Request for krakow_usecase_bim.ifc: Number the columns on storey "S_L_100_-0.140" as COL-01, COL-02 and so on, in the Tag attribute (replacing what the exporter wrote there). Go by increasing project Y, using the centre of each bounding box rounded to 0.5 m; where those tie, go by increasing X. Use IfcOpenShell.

First a look at what the model holds.

```python
import ifcopenshell
import ifcopenshell.util.element
import ifcopenshell.util.placement

model = ifcopenshell.open("krakow_usecase_bim.ifc")
print(model.schema)
storey = next(s for s in model.by_type("IfcBuildingStorey") if s.Name == "S_L_100_-0.140")
columns = [e for e in ifcopenshell.util.element.get_decomposition(storey) if e.is_a("IfcColumn")]
for e in sorted(columns, key=lambda e: e.id()):
    origin = ifcopenshell.util.placement.get_local_placement(e.ObjectPlacement)[:3, 3]
    print(e.id(), e.Tag, e.Name, origin.round(2) + 0.0, sep=" | ")
```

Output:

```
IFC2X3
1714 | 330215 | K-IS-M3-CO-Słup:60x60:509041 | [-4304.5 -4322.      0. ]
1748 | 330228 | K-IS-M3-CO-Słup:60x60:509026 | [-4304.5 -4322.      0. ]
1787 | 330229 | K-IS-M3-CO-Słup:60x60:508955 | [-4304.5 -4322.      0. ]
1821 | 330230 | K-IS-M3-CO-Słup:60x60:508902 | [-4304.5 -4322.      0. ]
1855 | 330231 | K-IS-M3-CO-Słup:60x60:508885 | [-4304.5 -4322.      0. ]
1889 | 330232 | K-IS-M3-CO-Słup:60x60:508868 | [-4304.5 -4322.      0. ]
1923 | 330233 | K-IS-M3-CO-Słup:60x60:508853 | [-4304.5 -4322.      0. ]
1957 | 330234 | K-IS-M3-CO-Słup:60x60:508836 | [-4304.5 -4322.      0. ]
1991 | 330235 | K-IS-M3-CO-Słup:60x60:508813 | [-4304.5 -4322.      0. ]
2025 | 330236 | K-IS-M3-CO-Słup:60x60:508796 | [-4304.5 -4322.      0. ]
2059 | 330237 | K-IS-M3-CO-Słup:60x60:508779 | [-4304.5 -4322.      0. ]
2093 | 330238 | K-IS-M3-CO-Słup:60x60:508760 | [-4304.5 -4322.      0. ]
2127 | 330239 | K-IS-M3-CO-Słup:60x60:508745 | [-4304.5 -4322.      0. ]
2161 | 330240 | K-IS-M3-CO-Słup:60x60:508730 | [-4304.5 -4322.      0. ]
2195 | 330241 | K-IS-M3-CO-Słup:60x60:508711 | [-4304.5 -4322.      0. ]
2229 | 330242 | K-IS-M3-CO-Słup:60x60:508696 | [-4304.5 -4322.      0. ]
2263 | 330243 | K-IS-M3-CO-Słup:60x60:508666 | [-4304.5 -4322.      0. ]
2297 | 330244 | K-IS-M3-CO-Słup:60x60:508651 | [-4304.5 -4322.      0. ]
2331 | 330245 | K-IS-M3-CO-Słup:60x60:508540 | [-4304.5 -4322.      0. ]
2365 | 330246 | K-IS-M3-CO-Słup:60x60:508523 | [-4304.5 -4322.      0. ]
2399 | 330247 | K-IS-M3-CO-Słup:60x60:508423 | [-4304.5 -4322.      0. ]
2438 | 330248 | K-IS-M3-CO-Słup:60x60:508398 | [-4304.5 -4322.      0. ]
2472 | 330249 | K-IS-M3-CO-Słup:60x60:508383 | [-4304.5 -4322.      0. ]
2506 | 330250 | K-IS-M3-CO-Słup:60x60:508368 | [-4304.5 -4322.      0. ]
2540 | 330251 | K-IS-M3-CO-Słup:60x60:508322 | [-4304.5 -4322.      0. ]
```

```python
import ifcopenshell
import ifcopenshell.geom
import ifcopenshell.util.element
import ifcopenshell.util.shape

model = ifcopenshell.open("krakow_usecase_bim.ifc")
settings = ifcopenshell.geom.settings()
settings.set("use-world-coords", True)


def centre(element):
    shape = ifcopenshell.geom.create_shape(settings, element)
    return ifcopenshell.util.shape.get_bbox_centroid(shape.geometry)


storey = next(s for s in model.by_type("IfcBuildingStorey") if s.Name == "S_L_100_-0.140")
columns = [e for e in ifcopenshell.util.element.get_decomposition(storey) if e.is_a("IfcColumn")]

# Insertion points can sit at a corner or the storey origin, so sort by the geometry (in metres).
centres = {e: centre(e) for e in columns}
columns.sort(key=lambda e: (round(centres[e][1] / 0.5), centres[e][0]))

for i, e in enumerate(columns, start=1):
    number = f"COL-{i:02d}"
    e.Tag = number
    print(e.id(), number)

model.write("krakow_usecase_bim_updated.ifc")
```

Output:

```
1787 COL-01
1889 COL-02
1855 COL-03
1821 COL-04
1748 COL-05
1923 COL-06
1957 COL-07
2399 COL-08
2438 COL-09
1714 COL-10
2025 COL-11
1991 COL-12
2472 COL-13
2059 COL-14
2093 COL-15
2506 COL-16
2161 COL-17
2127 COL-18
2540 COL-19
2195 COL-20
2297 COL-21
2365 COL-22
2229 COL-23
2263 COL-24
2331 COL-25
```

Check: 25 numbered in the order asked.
